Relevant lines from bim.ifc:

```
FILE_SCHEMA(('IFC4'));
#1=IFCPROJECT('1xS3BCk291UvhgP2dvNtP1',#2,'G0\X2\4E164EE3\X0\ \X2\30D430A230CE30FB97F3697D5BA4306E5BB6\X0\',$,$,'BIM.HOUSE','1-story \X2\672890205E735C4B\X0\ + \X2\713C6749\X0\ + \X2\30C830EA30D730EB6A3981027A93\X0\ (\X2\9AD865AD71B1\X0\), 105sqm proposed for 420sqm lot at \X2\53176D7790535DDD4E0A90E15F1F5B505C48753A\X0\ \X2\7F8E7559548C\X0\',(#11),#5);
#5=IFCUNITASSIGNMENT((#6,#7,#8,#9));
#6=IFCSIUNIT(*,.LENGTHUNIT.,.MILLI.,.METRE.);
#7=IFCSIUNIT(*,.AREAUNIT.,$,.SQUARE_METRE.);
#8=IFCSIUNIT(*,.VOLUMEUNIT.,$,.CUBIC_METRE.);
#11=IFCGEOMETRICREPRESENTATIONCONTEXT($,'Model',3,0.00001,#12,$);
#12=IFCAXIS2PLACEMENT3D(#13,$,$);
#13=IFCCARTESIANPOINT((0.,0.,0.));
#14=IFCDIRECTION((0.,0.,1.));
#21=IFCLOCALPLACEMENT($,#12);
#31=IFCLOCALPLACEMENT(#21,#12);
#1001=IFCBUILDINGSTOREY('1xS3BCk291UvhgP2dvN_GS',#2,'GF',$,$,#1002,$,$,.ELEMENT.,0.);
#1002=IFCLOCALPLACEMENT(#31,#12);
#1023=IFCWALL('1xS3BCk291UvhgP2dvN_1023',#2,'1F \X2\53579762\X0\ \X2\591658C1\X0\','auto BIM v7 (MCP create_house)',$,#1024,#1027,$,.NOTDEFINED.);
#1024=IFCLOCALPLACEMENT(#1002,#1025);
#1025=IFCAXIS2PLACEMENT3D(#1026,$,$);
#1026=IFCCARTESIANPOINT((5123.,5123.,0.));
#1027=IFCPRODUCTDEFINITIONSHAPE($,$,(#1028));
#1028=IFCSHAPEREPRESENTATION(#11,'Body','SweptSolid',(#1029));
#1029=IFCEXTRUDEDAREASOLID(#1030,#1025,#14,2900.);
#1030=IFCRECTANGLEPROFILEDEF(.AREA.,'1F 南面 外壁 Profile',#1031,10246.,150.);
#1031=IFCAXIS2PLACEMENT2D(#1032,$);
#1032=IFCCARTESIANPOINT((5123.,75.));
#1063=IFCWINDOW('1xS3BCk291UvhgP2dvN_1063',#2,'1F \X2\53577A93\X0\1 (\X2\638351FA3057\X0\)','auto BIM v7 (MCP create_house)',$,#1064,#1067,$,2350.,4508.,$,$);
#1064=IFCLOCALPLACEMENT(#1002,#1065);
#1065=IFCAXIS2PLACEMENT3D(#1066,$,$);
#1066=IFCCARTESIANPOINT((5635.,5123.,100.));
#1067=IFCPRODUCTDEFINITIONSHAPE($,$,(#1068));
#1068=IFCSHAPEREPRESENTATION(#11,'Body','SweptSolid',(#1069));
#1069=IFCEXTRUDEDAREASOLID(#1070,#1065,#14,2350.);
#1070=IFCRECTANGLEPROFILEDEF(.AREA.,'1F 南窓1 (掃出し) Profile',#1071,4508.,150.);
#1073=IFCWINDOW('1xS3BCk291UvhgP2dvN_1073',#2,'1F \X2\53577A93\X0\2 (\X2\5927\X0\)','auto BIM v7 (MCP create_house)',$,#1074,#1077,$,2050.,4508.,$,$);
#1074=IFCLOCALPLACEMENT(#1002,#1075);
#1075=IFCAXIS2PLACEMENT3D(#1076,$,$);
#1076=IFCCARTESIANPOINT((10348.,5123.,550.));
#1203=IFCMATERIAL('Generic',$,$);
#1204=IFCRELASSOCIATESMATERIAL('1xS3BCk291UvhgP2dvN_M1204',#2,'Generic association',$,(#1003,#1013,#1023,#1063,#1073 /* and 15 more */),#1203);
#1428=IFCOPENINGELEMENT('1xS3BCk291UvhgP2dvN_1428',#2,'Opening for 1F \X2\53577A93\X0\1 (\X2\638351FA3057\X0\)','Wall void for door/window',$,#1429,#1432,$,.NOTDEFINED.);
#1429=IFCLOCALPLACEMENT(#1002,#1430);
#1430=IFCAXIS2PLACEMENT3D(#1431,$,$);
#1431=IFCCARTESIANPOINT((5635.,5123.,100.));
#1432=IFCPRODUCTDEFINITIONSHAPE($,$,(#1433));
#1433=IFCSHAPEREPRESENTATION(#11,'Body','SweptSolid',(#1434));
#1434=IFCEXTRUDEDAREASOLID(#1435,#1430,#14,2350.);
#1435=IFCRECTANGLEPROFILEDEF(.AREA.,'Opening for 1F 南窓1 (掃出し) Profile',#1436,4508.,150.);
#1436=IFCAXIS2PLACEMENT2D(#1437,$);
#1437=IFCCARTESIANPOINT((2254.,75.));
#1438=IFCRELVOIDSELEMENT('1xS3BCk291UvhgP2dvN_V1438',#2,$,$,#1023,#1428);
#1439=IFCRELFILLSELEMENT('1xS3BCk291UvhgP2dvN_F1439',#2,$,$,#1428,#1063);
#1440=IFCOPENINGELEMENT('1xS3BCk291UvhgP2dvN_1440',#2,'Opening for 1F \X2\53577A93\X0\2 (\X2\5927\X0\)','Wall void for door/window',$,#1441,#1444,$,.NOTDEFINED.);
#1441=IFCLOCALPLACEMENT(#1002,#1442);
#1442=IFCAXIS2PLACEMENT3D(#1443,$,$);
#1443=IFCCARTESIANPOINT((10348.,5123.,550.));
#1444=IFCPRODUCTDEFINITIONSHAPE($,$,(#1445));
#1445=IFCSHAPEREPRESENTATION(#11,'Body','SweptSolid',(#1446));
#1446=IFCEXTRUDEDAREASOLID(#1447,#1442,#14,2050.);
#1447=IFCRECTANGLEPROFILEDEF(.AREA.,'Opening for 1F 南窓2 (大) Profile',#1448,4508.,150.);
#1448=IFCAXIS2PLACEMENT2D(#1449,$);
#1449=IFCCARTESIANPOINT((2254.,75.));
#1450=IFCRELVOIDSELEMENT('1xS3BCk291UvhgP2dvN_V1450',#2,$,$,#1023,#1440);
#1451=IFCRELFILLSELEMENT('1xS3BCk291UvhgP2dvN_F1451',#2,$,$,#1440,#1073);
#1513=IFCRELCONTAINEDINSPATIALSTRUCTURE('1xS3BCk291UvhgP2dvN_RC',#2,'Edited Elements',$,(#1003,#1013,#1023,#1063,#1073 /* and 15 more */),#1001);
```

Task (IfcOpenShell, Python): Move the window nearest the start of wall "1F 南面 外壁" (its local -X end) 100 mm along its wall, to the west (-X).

```python
import ifcopenshell
import ifcopenshell.api.geometry
import ifcopenshell.util.placement
import ifcopenshell.util.unit

model = ifcopenshell.open("bim.ifc")
unit_scale = ifcopenshell.util.unit.calculate_unit_scale(model)

window = model.by_guid("1xS3BCk291UvhgP2dvN_1063")
opening = window.FillsVoids[0].RelatingOpeningElement
wall = opening.VoidsElements[0].RelatingBuildingElement

wall_matrix = ifcopenshell.util.placement.get_local_placement(wall.ObjectPlacement)
shift = wall_matrix[:3, 0] * -0.1 / unit_scale
before = ifcopenshell.util.placement.get_local_placement(window.ObjectPlacement)[:3, 3].copy()

# The window is not placed relative to its opening, so move both.
for product in (opening, window):
    matrix = ifcopenshell.util.placement.get_local_placement(product.ObjectPlacement)
    matrix[:3, 3] += shift
    ifcopenshell.api.geometry.edit_object_placement(model, product=product, matrix=matrix, is_si=False)

after = ifcopenshell.util.placement.get_local_placement(window.ObjectPlacement)[:3, 3]
print("window moved by", (after - before).round(3) + 0.0)

model.write("bim_v2.ifc")
```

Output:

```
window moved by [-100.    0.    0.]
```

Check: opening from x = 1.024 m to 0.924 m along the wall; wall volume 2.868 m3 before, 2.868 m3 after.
